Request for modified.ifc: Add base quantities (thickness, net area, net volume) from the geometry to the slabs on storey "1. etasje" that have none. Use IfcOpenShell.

First a look at what the model holds.

```python
import ifcopenshell
import ifcopenshell.util.element
import ifcopenshell.util.unit

model = ifcopenshell.open("modified.ifc")
print(model.schema)
for unit_type in ("LENGTHUNIT", "AREAUNIT", "VOLUMEUNIT"):
    print(unit_type, ifcopenshell.util.unit.calculate_unit_scale(model, unit_type))
storey = next(s for s in model.by_type("IfcBuildingStorey") if s.Name == "1. etasje")
slabs = [e for e in ifcopenshell.util.element.get_decomposition(storey) if e.is_a("IfcSlab")]
for e in sorted(slabs, key=lambda e: e.id()):
    print(e.id(), e.is_a(), e.Name, list(ifcopenshell.util.element.get_psets(e, qtos_only=True)), sep=" | ")
```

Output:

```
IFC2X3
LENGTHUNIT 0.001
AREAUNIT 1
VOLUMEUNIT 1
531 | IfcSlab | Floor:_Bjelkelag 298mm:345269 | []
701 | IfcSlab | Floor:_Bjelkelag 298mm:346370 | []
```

```python
import ifcopenshell
import ifcopenshell.api.pset
import ifcopenshell.geom
import ifcopenshell.util.element
import ifcopenshell.util.shape
import ifcopenshell.util.unit

model = ifcopenshell.open("modified.ifc")
unit_scale = ifcopenshell.util.unit.calculate_unit_scale(model)
area_scale = ifcopenshell.util.unit.calculate_unit_scale(model, "AREAUNIT")
volume_scale = ifcopenshell.util.unit.calculate_unit_scale(model, "VOLUMEUNIT")
settings = ifcopenshell.geom.settings()

storey = next(s for s in model.by_type("IfcBuildingStorey") if s.Name == "1. etasje")
slabs = [e for e in ifcopenshell.util.element.get_decomposition(storey) if e.is_a("IfcSlab")]

for e in sorted(slabs, key=lambda e: e.id()):
    if ifcopenshell.util.element.get_psets(e, qtos_only=True, should_inherit=False):
        continue
    # Geometry comes back in metres, in the element's own axes.
    shape = ifcopenshell.geom.create_shape(settings, e)
    values = {
        "Width": ifcopenshell.util.shape.get_z(shape.geometry) / unit_scale,
        "NetArea": ifcopenshell.util.shape.get_footprint_area(shape.geometry) / area_scale,
        "NetVolume": ifcopenshell.util.shape.get_volume(shape.geometry) / volume_scale,
    }
    qto = ifcopenshell.api.pset.add_qto(model, product=e, name="BaseQuantities")
    ifcopenshell.api.pset.edit_qto(model, qto=qto, properties=values)
    print(e.id(), {k: round(v, 3) for k, v in values.items()})

model.write("modified_rev.ifc")
```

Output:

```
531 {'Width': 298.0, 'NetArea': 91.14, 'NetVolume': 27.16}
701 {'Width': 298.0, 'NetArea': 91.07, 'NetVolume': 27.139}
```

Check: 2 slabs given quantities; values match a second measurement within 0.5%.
